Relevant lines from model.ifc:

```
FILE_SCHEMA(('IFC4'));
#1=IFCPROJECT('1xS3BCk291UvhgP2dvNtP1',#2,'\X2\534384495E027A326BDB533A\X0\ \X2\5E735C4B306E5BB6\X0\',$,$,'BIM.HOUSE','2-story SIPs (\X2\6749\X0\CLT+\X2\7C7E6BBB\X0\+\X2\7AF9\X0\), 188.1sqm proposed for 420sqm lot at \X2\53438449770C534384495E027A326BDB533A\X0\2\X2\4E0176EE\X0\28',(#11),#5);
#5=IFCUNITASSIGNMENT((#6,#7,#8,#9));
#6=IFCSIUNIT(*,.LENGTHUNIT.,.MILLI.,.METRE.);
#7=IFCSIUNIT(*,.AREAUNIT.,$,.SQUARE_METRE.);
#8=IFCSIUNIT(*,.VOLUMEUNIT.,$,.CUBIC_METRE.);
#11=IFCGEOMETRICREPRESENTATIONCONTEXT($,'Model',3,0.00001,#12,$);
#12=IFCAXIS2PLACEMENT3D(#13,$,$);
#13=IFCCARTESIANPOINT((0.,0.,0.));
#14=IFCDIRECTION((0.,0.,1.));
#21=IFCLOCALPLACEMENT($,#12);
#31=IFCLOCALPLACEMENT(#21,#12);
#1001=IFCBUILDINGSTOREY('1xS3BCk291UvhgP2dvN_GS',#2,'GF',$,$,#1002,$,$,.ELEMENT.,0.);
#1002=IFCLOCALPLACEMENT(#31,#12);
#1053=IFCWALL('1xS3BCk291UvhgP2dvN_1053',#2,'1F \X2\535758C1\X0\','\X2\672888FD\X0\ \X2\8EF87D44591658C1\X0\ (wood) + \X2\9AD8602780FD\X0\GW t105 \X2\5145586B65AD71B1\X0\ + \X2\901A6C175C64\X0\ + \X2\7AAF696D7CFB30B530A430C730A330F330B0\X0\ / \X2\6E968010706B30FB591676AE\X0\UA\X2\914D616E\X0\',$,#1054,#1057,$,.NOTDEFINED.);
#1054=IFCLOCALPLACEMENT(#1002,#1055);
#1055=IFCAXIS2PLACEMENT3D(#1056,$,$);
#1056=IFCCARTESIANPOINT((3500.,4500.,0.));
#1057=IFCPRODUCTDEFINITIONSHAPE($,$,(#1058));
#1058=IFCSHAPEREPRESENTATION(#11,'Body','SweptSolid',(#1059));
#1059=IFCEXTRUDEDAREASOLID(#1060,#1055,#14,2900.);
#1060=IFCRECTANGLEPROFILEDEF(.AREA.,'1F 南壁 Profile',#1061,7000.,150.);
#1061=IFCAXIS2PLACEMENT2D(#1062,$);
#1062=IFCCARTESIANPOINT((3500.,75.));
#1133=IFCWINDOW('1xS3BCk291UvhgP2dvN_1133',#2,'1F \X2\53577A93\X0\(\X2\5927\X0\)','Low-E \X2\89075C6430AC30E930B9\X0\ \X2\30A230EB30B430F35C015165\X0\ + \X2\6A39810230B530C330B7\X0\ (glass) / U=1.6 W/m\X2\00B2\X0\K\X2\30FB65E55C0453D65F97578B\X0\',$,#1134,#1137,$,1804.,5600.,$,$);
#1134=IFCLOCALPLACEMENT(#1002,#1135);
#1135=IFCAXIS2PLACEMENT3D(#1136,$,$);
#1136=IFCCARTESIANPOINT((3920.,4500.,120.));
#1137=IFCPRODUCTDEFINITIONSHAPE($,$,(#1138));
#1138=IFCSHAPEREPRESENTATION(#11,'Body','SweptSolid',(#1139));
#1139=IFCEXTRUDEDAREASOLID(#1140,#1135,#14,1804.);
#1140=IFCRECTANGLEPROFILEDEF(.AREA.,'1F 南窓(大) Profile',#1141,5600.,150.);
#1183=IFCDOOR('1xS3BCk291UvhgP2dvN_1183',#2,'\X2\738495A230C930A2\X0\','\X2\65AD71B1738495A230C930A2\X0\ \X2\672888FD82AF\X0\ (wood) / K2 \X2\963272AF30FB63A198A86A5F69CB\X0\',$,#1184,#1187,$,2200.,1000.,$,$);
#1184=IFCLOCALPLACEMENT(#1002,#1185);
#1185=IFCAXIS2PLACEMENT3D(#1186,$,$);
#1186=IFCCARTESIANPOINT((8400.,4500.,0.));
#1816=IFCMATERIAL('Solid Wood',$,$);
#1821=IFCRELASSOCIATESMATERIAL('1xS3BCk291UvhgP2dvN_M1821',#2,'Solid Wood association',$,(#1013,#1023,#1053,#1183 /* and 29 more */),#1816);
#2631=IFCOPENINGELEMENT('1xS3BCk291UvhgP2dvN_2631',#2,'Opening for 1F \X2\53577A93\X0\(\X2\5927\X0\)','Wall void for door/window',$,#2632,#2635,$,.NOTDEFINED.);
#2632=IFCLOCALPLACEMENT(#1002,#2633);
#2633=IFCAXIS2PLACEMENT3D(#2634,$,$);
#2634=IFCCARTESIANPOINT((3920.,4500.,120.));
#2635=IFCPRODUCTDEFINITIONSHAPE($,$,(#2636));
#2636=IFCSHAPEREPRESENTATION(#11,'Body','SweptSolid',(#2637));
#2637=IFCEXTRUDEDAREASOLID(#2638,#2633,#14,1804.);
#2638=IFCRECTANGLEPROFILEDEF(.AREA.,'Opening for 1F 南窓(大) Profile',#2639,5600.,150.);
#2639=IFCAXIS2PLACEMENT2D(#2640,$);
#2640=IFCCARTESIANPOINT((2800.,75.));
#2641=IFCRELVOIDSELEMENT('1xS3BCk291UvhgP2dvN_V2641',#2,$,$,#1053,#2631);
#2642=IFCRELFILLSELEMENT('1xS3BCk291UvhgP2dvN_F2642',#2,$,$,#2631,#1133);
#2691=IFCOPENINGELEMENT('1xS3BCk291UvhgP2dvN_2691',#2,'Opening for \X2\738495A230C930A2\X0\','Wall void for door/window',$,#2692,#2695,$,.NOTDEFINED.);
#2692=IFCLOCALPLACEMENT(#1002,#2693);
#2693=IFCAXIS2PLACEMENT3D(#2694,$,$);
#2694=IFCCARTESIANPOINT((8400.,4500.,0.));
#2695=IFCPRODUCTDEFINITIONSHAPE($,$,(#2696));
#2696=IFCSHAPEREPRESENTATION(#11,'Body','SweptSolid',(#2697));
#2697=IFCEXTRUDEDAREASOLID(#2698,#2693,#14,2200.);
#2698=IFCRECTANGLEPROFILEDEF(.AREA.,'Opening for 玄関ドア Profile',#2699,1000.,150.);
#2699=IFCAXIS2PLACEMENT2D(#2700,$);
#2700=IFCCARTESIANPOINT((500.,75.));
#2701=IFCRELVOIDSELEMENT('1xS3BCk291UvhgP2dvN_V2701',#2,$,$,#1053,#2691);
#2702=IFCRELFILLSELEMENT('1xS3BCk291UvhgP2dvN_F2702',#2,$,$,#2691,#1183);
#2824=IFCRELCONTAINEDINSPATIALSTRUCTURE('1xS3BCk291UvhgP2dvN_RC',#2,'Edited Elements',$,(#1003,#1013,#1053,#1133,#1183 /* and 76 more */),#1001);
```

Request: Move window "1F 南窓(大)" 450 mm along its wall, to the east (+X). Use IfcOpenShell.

```python
import ifcopenshell
import ifcopenshell.api.geometry
import ifcopenshell.util.placement
import ifcopenshell.util.unit

model = ifcopenshell.open("model.ifc")
unit_scale = ifcopenshell.util.unit.calculate_unit_scale(model)

window = model.by_id(1133)
opening = window.FillsVoids[0].RelatingOpeningElement
wall = opening.VoidsElements[0].RelatingBuildingElement

wall_matrix = ifcopenshell.util.placement.get_local_placement(wall.ObjectPlacement)
shift = wall_matrix[:3, 0] * 0.45 / unit_scale
before = ifcopenshell.util.placement.get_local_placement(window.ObjectPlacement)[:3, 3].copy()

# The window is not placed relative to its opening, so move both.
for product in (opening, window):
    matrix = ifcopenshell.util.placement.get_local_placement(product.ObjectPlacement)
    matrix[:3, 3] += shift
    ifcopenshell.api.geometry.edit_object_placement(model, product=product, matrix=matrix, is_si=False)

after = ifcopenshell.util.placement.get_local_placement(window.ObjectPlacement)[:3, 3]
print("window moved by", (after - before).round(3) + 0.0)

model.write("model_v2.ifc")
```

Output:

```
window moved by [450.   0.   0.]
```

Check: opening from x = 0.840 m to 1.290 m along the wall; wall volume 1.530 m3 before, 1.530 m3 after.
